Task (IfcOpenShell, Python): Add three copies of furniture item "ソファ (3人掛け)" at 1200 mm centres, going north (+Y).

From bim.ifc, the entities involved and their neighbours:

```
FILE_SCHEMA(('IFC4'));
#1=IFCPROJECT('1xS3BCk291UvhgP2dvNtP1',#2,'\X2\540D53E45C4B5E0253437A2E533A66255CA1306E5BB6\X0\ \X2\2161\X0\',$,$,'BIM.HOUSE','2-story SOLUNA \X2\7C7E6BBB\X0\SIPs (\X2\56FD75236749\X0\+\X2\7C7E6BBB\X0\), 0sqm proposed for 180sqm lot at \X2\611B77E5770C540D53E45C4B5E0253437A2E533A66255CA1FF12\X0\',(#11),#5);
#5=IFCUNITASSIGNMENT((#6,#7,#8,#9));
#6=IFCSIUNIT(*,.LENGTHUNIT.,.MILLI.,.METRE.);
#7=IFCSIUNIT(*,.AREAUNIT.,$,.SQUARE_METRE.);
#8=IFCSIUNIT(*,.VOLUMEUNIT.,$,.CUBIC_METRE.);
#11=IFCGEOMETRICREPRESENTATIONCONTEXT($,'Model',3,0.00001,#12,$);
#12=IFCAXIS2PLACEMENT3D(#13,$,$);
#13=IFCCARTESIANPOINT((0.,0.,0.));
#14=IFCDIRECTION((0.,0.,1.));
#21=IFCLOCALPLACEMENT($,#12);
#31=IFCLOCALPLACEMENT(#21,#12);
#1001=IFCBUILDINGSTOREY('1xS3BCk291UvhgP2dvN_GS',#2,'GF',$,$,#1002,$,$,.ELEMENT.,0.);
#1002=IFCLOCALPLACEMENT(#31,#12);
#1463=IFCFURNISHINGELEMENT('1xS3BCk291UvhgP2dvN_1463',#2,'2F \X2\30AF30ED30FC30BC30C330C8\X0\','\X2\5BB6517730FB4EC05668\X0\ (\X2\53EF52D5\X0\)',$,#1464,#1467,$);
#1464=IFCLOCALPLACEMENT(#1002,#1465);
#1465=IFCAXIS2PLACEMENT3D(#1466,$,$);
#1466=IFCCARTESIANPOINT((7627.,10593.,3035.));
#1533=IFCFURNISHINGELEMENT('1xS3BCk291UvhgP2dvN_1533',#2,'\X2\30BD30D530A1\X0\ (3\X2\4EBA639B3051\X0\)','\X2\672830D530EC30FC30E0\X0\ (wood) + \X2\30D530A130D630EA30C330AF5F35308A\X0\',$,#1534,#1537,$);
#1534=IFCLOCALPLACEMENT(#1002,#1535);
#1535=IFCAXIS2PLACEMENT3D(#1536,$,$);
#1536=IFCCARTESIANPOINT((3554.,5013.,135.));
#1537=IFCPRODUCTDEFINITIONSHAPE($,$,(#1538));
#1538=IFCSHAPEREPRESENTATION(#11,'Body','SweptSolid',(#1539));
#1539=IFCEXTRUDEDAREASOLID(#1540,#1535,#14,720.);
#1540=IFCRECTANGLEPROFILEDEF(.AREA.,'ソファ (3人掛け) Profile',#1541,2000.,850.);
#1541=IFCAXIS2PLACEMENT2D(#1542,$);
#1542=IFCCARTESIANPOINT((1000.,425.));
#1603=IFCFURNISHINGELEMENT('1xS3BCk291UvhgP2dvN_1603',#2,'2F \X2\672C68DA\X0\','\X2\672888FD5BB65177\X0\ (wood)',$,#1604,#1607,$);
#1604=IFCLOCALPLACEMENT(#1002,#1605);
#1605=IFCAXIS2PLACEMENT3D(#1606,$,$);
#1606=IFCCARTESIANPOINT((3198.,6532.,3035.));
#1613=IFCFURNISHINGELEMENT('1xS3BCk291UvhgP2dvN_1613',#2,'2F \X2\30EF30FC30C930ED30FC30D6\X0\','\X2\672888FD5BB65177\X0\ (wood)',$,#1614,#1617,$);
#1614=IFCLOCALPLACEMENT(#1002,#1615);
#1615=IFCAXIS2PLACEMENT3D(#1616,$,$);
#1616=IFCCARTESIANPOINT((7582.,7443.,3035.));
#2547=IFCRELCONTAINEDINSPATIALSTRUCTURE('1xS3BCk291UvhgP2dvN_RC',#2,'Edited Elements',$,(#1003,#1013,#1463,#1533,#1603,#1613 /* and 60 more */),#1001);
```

```python
import numpy as np
import ifcopenshell
import ifcopenshell.api.geometry
import ifcopenshell.api.root
import ifcopenshell.util.element
import ifcopenshell.util.placement

model = ifcopenshell.open("bim.ifc")


def reuse_history(source, copy):
    """copy_class also copies each property set's owner history, people and application; keep the originals."""
    for rel in copy.IsDefinedBy:
        if rel.is_a("IfcRelDefinesByProperties") and (history := rel.RelatingPropertyDefinition.OwnerHistory):
            rel.RelatingPropertyDefinition.OwnerHistory = source.OwnerHistory
            ifcopenshell.util.element.remove_deep2(model, history)


source = model.by_guid("1xS3BCk291UvhgP2dvN_1533")
base = ifcopenshell.util.placement.get_local_placement(source.ObjectPlacement)
step = np.array([0.0, 1.0, 0.0]) * 1200.0

for i in range(1, 4):
    copy = ifcopenshell.api.root.copy_class(model, product=source)
    copy.Representation = ifcopenshell.util.element.copy_deep(
        model, source.Representation, exclude=["IfcGeometricRepresentationContext", "IfcRepresentationMap"]
    )
    reuse_history(source, copy)
    matrix = base.copy()
    matrix[:3, 3] += i * step
    print("added at", matrix[:3, 3].round(3) + 0.0)
    ifcopenshell.api.geometry.edit_object_placement(model, product=copy, matrix=matrix, is_si=False)

model.write("bim_edited.ifc")
```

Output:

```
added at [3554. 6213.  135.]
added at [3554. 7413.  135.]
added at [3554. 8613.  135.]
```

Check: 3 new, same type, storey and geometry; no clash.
